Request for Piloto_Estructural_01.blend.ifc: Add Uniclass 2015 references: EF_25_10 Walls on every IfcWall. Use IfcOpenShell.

First a look at what the model holds.

```python
import ifcopenshell

model = ifcopenshell.open("Piloto_Estructural_01.blend.ifc")
print(model.schema)
print("classifications:", [c.Name for c in model.by_type("IfcClassification")])
for ifc_class in ("IfcDoor", "IfcRoof", "IfcStair", "IfcWall", "IfcWindow"):
    print(ifc_class, len(model.by_type(ifc_class)))
```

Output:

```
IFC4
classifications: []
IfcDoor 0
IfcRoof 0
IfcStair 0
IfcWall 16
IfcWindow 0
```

```python
import ifcopenshell
import ifcopenshell.api.classification

model = ifcopenshell.open("Piloto_Estructural_01.blend.ifc")

system = ifcopenshell.api.classification.add_classification(model, classification="Uniclass 2015")

codes = {
    "IfcWall": ("EF_25_10", "Walls"),
}
for ifc_class, (code, name) in codes.items():
    products = model.by_type(ifc_class)
    ifcopenshell.api.classification.add_reference(
        model, products=products, classification=system, identification=code, name=name
    )
    print(code, len(products))

model.write("Piloto_Estructural_01.blend-out.ifc")
```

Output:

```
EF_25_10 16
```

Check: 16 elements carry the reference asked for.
